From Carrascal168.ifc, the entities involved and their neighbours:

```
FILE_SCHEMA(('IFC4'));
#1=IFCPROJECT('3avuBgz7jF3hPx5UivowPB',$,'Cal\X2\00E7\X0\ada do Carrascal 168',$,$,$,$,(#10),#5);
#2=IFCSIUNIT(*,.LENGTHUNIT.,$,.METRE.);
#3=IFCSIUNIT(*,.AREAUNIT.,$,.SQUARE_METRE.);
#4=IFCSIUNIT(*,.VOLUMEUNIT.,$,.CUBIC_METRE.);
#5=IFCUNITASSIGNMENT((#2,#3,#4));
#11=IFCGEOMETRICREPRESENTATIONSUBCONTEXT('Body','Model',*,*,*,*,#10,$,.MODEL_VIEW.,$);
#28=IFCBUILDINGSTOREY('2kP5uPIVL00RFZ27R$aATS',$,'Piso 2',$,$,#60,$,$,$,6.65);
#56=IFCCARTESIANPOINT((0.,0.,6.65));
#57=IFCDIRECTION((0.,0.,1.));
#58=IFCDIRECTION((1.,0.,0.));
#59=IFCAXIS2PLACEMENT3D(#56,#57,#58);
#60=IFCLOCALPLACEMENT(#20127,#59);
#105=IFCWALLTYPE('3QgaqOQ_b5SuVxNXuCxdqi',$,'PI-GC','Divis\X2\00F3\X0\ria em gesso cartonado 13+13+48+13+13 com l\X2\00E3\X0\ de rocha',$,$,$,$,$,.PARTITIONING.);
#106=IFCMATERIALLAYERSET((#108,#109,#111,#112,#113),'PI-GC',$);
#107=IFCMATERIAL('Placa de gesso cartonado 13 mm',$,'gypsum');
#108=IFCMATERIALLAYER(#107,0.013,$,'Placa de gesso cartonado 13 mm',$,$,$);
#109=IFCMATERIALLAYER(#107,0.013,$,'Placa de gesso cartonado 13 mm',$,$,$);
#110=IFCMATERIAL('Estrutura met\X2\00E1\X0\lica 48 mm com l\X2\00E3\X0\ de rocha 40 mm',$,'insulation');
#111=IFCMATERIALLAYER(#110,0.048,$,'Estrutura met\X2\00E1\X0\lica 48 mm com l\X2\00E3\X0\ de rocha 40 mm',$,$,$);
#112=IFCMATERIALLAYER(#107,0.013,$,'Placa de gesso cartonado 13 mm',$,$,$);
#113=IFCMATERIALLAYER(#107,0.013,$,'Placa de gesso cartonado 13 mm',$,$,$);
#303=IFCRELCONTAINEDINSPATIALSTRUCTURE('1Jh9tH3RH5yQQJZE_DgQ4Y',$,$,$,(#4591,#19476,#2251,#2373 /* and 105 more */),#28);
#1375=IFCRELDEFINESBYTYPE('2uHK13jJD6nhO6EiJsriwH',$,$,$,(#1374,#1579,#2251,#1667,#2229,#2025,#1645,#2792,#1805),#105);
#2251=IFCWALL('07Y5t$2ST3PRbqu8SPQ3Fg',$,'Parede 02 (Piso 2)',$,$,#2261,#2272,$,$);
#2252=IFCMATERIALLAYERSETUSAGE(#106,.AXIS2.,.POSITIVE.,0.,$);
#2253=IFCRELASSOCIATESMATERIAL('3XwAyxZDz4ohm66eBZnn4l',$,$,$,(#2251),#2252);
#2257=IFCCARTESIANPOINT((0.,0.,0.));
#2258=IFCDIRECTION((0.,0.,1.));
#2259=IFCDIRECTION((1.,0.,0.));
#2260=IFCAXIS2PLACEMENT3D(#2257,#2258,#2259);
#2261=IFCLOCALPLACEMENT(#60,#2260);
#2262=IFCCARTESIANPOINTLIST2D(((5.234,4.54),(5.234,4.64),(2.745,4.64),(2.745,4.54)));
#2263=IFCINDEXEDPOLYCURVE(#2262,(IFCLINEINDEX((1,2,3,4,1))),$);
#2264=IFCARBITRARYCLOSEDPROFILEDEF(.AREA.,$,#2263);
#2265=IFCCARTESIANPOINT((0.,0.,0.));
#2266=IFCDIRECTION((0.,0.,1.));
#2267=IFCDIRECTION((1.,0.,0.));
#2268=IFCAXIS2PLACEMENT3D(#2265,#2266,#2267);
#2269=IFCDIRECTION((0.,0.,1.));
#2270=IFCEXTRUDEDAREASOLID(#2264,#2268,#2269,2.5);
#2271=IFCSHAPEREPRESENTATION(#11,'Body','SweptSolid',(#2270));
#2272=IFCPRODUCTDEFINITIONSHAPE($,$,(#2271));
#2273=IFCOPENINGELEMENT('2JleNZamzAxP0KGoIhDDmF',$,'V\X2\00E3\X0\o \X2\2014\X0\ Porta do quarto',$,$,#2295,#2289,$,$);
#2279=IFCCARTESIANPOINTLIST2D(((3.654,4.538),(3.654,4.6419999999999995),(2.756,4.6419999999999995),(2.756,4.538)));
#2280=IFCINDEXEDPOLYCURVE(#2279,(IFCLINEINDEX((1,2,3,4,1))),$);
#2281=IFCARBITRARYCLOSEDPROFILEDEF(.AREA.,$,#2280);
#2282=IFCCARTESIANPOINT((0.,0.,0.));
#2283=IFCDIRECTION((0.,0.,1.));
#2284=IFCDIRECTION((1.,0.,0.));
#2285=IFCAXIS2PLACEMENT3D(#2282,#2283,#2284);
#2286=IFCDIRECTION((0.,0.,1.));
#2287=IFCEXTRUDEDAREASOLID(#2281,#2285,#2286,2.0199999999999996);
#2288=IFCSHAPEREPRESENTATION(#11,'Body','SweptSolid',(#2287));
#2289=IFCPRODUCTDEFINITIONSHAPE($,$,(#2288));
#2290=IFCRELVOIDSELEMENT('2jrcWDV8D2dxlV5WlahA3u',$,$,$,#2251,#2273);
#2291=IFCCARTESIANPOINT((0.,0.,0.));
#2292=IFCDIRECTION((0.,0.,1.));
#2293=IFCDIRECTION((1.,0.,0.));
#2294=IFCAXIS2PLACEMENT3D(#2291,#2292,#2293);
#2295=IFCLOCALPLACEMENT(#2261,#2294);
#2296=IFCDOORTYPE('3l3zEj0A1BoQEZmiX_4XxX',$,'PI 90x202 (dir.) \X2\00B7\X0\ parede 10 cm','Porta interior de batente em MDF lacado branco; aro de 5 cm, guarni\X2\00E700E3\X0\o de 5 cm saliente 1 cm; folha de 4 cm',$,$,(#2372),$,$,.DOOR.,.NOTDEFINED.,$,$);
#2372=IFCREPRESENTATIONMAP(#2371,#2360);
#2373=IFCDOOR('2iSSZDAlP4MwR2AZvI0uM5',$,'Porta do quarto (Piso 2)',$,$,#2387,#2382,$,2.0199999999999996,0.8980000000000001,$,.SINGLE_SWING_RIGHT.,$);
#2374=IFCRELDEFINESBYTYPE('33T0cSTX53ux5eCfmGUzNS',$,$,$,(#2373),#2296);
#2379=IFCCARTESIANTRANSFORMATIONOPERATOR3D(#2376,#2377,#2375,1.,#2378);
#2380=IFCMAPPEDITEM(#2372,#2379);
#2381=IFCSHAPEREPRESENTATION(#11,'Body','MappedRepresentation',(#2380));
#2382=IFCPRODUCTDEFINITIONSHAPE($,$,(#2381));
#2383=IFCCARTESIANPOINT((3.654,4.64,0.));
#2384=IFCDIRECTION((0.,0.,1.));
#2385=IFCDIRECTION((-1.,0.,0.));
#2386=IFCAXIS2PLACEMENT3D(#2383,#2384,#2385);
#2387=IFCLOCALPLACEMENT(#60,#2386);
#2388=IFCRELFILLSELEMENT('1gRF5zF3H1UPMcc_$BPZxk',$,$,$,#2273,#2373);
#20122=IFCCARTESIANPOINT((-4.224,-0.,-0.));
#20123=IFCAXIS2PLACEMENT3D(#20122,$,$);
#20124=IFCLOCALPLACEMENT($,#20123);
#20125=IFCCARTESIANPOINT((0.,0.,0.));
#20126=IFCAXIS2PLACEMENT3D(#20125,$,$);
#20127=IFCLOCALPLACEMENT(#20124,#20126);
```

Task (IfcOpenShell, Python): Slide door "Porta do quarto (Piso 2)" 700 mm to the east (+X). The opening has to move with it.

```python
import ifcopenshell
import ifcopenshell.api.geometry
import ifcopenshell.util.placement
import ifcopenshell.util.unit

model = ifcopenshell.open("Carrascal168.ifc")
unit_scale = ifcopenshell.util.unit.calculate_unit_scale(model)

door = model.by_id(2373)
opening = door.FillsVoids[0].RelatingOpeningElement
wall = opening.VoidsElements[0].RelatingBuildingElement

wall_matrix = ifcopenshell.util.placement.get_local_placement(wall.ObjectPlacement)
shift = wall_matrix[:3, 0] * 0.7 / unit_scale
before = ifcopenshell.util.placement.get_local_placement(door.ObjectPlacement)[:3, 3].copy()

# The door is not placed relative to its opening, so move both.
for product in (opening, door):
    matrix = ifcopenshell.util.placement.get_local_placement(product.ObjectPlacement)
    matrix[:3, 3] += shift
    ifcopenshell.api.geometry.edit_object_placement(model, product=product, matrix=matrix, is_si=False)

after = ifcopenshell.util.placement.get_local_placement(door.ObjectPlacement)[:3, 3]
print("door moved by", (after - before).round(3) + 0.0)

model.write("Carrascal168_v2.ifc")
```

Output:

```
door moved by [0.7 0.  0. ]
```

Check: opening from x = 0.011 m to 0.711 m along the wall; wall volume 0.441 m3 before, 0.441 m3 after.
